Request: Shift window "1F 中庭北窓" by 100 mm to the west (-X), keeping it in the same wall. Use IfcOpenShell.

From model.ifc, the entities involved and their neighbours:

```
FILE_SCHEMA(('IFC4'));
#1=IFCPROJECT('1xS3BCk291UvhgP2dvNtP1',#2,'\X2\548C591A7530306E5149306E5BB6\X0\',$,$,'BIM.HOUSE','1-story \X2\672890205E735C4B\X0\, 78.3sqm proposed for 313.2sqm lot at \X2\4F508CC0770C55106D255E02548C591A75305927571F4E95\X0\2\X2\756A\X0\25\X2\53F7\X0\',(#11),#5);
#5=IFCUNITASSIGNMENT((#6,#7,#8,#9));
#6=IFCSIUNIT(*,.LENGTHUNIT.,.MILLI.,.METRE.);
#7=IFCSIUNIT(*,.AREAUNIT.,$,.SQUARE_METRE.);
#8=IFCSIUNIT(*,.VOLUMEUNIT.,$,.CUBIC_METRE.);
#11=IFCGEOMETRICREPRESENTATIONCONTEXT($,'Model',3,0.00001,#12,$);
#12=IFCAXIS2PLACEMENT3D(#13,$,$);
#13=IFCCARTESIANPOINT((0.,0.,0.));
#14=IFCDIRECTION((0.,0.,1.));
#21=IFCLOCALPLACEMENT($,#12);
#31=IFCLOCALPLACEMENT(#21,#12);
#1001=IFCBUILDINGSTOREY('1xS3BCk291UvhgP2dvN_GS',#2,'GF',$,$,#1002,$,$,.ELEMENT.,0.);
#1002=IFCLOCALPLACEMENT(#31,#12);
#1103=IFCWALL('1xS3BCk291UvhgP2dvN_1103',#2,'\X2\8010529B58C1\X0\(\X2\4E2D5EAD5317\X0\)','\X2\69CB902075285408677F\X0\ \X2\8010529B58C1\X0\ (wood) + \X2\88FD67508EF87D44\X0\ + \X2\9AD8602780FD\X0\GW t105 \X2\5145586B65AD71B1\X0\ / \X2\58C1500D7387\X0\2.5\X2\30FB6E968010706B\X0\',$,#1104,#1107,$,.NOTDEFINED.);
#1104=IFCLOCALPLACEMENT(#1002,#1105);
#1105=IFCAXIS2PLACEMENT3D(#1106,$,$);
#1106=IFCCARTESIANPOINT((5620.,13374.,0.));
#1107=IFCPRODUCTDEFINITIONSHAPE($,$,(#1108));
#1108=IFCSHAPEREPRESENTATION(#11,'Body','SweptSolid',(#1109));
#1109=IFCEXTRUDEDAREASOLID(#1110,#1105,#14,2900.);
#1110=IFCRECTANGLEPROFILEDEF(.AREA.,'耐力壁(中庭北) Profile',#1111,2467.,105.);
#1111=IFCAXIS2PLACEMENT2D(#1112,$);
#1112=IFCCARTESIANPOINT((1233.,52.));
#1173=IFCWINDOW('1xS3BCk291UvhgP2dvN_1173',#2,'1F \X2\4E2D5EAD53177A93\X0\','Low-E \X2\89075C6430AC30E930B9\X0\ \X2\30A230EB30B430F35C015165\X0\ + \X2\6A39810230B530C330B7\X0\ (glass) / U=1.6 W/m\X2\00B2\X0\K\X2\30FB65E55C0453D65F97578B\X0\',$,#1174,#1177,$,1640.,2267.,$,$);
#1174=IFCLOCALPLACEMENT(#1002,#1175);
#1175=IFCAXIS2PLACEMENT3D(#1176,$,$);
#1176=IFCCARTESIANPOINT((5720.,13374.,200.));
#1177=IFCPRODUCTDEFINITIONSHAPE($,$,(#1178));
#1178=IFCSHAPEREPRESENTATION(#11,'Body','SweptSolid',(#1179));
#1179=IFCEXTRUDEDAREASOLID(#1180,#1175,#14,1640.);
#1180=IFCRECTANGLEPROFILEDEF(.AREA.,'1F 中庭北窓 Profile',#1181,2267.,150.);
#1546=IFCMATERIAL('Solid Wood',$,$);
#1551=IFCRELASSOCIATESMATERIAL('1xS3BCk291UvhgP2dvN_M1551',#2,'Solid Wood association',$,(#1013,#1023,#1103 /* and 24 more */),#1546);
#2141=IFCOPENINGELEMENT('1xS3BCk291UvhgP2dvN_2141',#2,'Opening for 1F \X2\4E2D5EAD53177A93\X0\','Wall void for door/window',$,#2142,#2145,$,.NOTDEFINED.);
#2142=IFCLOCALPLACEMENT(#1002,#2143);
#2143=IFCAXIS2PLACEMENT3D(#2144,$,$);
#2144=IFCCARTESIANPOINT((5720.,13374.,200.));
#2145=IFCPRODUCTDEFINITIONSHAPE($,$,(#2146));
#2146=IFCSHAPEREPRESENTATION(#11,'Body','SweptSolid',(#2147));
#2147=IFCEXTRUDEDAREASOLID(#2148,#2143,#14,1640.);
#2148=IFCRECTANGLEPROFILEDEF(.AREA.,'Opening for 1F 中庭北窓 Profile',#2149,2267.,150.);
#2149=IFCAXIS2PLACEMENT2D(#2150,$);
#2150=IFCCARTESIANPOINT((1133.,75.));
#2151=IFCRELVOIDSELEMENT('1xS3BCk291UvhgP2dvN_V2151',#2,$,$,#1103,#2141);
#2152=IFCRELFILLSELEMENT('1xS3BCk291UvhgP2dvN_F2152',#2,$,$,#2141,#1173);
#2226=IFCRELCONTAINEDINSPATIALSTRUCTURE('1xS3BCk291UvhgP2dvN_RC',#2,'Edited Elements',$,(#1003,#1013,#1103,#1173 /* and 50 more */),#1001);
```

```python
import ifcopenshell
import ifcopenshell.api.geometry
import ifcopenshell.util.placement
import ifcopenshell.util.unit

model = ifcopenshell.open("model.ifc")
unit_scale = ifcopenshell.util.unit.calculate_unit_scale(model)

window = model.by_guid("1xS3BCk291UvhgP2dvN_1173")
opening = window.FillsVoids[0].RelatingOpeningElement
wall = opening.VoidsElements[0].RelatingBuildingElement

wall_matrix = ifcopenshell.util.placement.get_local_placement(wall.ObjectPlacement)
shift = wall_matrix[:3, 0] * -0.1 / unit_scale
before = ifcopenshell.util.placement.get_local_placement(window.ObjectPlacement)[:3, 3].copy()

# The window is not placed relative to its opening, so move both.
for product in (opening, window):
    matrix = ifcopenshell.util.placement.get_local_placement(product.ObjectPlacement)
    matrix[:3, 3] += shift
    ifcopenshell.api.geometry.edit_object_placement(model, product=product, matrix=matrix, is_si=False)

after = ifcopenshell.util.placement.get_local_placement(window.ObjectPlacement)[:3, 3]
print("window moved by", (after - before).round(3) + 0.0)

model.write("model_rev.ifc")
```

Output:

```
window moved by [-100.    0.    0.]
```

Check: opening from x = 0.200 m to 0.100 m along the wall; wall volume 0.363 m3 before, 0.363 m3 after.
